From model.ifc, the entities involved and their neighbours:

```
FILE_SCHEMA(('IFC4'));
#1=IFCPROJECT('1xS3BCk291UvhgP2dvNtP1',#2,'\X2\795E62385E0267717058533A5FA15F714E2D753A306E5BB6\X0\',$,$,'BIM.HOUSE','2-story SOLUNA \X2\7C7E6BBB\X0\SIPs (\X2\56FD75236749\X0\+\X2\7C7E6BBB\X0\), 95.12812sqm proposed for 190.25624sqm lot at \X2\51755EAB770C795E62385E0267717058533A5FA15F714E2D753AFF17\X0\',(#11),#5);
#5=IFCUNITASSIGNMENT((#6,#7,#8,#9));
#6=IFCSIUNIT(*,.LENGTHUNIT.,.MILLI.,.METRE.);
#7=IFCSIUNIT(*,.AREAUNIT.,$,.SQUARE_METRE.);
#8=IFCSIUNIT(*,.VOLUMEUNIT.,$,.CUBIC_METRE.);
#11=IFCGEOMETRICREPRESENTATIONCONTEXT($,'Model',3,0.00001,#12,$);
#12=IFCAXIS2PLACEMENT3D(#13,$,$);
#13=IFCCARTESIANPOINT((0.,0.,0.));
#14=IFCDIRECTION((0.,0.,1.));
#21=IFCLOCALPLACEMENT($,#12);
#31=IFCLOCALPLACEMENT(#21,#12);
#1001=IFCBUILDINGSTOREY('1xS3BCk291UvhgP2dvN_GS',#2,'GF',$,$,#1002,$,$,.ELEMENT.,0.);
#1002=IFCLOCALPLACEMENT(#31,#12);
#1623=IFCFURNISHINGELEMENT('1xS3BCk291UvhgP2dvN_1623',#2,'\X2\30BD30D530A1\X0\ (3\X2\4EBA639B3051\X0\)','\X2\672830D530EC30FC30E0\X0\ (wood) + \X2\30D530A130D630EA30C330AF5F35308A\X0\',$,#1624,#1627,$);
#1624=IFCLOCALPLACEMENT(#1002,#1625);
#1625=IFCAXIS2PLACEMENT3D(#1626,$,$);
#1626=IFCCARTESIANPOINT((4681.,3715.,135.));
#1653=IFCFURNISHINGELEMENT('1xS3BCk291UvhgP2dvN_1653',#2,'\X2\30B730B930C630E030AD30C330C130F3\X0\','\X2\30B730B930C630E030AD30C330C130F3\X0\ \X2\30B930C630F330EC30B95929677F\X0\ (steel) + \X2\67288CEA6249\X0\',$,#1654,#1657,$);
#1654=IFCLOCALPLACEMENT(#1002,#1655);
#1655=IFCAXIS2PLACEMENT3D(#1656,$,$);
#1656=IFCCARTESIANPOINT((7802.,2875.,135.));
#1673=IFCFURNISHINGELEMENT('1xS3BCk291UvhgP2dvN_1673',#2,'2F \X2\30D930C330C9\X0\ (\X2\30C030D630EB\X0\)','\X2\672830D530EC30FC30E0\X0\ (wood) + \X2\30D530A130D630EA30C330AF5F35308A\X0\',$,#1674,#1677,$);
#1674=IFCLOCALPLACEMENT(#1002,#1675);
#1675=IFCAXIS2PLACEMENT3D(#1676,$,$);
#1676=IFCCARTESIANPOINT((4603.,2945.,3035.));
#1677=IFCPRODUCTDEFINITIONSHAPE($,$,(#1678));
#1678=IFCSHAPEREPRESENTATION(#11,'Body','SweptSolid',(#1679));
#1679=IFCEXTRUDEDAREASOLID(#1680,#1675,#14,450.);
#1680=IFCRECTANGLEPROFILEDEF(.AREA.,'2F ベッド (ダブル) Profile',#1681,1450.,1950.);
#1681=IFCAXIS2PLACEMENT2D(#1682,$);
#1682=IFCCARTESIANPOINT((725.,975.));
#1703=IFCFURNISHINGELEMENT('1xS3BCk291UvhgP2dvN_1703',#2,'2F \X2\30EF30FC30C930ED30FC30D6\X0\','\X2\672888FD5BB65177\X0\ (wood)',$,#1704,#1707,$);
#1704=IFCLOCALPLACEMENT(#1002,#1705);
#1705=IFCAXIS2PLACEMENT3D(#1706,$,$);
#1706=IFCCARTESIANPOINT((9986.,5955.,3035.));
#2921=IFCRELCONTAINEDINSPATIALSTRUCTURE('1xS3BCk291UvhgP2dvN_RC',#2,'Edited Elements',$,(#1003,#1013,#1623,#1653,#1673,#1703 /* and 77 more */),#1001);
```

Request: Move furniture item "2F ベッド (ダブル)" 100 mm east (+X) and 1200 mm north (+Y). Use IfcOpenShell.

```python
import ifcopenshell
import ifcopenshell.api.geometry
import ifcopenshell.util.placement

model = ifcopenshell.open("model.ifc")

item = model.by_guid("1xS3BCk291UvhgP2dvN_1673")
matrix = ifcopenshell.util.placement.get_local_placement(item.ObjectPlacement)
matrix[0, 3] += 100.0
matrix[1, 3] += 1200.0
ifcopenshell.api.geometry.edit_object_placement(model, product=item, matrix=matrix, is_si=False)

print(ifcopenshell.util.placement.get_local_placement(item.ObjectPlacement).round(3) + 0.0)

model.write("model_edited.ifc")
```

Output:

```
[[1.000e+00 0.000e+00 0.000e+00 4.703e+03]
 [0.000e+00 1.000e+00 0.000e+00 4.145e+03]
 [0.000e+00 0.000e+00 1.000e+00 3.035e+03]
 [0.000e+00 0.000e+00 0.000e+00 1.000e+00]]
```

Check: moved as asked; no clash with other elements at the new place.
